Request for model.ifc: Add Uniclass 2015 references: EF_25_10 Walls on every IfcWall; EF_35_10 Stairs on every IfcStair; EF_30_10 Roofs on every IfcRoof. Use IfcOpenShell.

First a look at what the model holds.

```python
import ifcopenshell

model = ifcopenshell.open("model.ifc")
print(model.schema)
print("classifications:", [c.Name for c in model.by_type("IfcClassification")])
for ifc_class in ("IfcDoor", "IfcRoof", "IfcStair", "IfcWall", "IfcWindow"):
    print(ifc_class, len(model.by_type(ifc_class)))
```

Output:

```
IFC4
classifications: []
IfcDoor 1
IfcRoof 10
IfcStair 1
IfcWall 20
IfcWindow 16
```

```python
import ifcopenshell
import ifcopenshell.api.classification

model = ifcopenshell.open("model.ifc")

system = ifcopenshell.api.classification.add_classification(model, classification="Uniclass 2015")

codes = {
    "IfcWall": ("EF_25_10", "Walls"),
    "IfcStair": ("EF_35_10", "Stairs"),
    "IfcRoof": ("EF_30_10", "Roofs"),
}
for ifc_class, (code, name) in codes.items():
    products = model.by_type(ifc_class)
    ifcopenshell.api.classification.add_reference(
        model, products=products, classification=system, identification=code, name=name
    )
    print(code, len(products))

model.write("model_rev.ifc")
```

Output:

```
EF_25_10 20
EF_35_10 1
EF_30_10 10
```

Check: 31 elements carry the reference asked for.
